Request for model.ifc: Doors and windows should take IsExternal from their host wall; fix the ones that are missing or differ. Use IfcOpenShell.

First a look at what the model holds.

```python
import ifcopenshell
import ifcopenshell.util.element

model = ifcopenshell.open("model.ifc")
print(model.schema)
seen = {}
for e in model.by_type("IfcDoor") + model.by_type("IfcWindow"):
    if not e.FillsVoids:
        continue
    host = e.FillsVoids[0].RelatingOpeningElement.VoidsElements[0].RelatingBuildingElement
    own = ifcopenshell.util.element.get_pset(e, f"Pset_{e.is_a()[3:].removesuffix('StandardCase')}Common", "IsExternal")
    wall = ifcopenshell.util.element.get_pset(host, "Pset_WallCommon", "IsExternal")
    seen[e.is_a(), own, wall] = seen.get((e.is_a(), own, wall), 0) + 1
for (cls, own, wall), count in sorted(seen.items(), key=str):
    print(count, cls, "IsExternal:", own, "| host wall:", wall)
```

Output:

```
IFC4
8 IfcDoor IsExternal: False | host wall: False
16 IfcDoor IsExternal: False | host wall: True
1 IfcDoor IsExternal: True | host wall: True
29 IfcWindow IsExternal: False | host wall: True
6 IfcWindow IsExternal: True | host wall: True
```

```python
import ifcopenshell
import ifcopenshell.api.pset
import ifcopenshell.util.element

model = ifcopenshell.open("model.ifc")

count = 0
for ifc_class, pset_name in (("IfcDoor", "Pset_DoorCommon"), ("IfcWindow", "Pset_WindowCommon")):
    for e in model.by_type(ifc_class):
        if not e.FillsVoids:
            continue
        host = e.FillsVoids[0].RelatingOpeningElement.VoidsElements[0].RelatingBuildingElement
        external = ifcopenshell.util.element.get_pset(host, "Pset_WallCommon", "IsExternal")
        if external is None or ifcopenshell.util.element.get_pset(e, pset_name, "IsExternal") == external:
            continue
        pset = ifcopenshell.api.pset.add_pset(model, product=e, name=pset_name)
        ifcopenshell.api.pset.edit_pset(model, pset=pset, properties={"IsExternal": external})
        count += 1

print(count, "updated")

model.write("model_v2.ifc")
```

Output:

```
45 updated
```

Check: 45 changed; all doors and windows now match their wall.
